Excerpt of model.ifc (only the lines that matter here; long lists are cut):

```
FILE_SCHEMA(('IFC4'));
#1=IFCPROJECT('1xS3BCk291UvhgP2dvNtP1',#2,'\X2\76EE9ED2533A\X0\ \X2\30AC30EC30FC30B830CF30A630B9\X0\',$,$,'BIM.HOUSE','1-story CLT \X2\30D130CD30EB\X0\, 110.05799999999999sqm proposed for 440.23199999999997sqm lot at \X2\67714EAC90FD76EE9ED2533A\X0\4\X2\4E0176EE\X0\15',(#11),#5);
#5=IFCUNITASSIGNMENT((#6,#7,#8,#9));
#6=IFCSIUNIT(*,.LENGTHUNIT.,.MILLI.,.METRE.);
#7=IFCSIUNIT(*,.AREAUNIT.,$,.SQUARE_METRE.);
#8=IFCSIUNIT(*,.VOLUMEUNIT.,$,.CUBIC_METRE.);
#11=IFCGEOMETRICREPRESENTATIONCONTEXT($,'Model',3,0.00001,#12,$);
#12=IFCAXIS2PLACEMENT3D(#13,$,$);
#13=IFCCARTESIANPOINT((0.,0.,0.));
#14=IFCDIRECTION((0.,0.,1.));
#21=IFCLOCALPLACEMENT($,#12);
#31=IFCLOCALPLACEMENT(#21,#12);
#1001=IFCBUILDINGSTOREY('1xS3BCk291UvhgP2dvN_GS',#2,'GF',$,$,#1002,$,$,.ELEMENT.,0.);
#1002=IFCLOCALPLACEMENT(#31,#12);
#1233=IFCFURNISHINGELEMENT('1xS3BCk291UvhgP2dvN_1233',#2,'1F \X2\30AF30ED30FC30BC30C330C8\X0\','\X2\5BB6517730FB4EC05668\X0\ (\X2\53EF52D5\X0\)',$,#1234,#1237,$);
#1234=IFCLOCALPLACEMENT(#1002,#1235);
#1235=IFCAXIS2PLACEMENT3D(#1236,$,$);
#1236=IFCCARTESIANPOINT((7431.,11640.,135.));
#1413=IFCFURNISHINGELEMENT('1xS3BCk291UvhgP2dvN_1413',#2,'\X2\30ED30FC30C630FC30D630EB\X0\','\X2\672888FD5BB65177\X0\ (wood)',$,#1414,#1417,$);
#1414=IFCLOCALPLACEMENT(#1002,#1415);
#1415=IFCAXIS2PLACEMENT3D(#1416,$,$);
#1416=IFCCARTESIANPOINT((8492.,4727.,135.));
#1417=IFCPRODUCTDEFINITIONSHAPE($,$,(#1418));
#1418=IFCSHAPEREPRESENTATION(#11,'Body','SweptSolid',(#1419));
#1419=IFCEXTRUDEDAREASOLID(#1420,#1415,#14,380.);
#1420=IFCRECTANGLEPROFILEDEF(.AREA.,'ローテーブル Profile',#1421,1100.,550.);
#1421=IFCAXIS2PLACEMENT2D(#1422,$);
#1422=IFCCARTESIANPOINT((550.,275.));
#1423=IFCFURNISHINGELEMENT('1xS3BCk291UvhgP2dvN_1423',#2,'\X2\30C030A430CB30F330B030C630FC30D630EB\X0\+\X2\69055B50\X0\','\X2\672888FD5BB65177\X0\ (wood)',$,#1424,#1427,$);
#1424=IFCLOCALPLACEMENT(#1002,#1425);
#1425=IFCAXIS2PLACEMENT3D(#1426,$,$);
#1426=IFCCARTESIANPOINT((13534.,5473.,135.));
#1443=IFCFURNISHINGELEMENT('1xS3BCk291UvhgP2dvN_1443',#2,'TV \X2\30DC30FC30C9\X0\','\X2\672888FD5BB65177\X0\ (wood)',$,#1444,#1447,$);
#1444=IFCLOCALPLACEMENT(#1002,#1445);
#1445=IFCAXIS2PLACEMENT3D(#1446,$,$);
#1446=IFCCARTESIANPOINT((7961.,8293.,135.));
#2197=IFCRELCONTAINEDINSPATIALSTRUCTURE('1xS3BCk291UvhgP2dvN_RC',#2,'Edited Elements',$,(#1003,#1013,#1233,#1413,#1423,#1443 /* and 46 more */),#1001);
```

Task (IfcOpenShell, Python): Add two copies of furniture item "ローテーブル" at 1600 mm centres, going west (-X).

```python
import numpy as np
import ifcopenshell
import ifcopenshell.api.geometry
import ifcopenshell.api.root
import ifcopenshell.util.element
import ifcopenshell.util.placement
import ifcopenshell.util.unit

model = ifcopenshell.open("model.ifc")
unit_scale = ifcopenshell.util.unit.calculate_unit_scale(model)


def reuse_history(source, copy):
    """copy_class also copies each property set's owner history, people and application; keep the originals."""
    for rel in copy.IsDefinedBy:
        if rel.is_a("IfcRelDefinesByProperties") and (history := rel.RelatingPropertyDefinition.OwnerHistory):
            rel.RelatingPropertyDefinition.OwnerHistory = source.OwnerHistory
            ifcopenshell.util.element.remove_deep2(model, history)


source = model.by_guid("1xS3BCk291UvhgP2dvN_1413")
base = ifcopenshell.util.placement.get_local_placement(source.ObjectPlacement)
step = np.array([-1.0, 0.0, 0.0]) * 1.6 / unit_scale

for i in range(1, 3):
    copy = ifcopenshell.api.root.copy_class(model, product=source)
    copy.Representation = ifcopenshell.util.element.copy_deep(
        model, source.Representation, exclude=["IfcGeometricRepresentationContext", "IfcRepresentationMap"]
    )
    reuse_history(source, copy)
    matrix = base.copy()
    matrix[:3, 3] += i * step
    print("added at", matrix[:3, 3].round(3) + 0.0)
    ifcopenshell.api.geometry.edit_object_placement(model, product=copy, matrix=matrix, is_si=False)

model.write("model_updated.ifc")
```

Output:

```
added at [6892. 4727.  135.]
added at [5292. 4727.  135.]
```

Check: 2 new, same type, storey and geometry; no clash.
